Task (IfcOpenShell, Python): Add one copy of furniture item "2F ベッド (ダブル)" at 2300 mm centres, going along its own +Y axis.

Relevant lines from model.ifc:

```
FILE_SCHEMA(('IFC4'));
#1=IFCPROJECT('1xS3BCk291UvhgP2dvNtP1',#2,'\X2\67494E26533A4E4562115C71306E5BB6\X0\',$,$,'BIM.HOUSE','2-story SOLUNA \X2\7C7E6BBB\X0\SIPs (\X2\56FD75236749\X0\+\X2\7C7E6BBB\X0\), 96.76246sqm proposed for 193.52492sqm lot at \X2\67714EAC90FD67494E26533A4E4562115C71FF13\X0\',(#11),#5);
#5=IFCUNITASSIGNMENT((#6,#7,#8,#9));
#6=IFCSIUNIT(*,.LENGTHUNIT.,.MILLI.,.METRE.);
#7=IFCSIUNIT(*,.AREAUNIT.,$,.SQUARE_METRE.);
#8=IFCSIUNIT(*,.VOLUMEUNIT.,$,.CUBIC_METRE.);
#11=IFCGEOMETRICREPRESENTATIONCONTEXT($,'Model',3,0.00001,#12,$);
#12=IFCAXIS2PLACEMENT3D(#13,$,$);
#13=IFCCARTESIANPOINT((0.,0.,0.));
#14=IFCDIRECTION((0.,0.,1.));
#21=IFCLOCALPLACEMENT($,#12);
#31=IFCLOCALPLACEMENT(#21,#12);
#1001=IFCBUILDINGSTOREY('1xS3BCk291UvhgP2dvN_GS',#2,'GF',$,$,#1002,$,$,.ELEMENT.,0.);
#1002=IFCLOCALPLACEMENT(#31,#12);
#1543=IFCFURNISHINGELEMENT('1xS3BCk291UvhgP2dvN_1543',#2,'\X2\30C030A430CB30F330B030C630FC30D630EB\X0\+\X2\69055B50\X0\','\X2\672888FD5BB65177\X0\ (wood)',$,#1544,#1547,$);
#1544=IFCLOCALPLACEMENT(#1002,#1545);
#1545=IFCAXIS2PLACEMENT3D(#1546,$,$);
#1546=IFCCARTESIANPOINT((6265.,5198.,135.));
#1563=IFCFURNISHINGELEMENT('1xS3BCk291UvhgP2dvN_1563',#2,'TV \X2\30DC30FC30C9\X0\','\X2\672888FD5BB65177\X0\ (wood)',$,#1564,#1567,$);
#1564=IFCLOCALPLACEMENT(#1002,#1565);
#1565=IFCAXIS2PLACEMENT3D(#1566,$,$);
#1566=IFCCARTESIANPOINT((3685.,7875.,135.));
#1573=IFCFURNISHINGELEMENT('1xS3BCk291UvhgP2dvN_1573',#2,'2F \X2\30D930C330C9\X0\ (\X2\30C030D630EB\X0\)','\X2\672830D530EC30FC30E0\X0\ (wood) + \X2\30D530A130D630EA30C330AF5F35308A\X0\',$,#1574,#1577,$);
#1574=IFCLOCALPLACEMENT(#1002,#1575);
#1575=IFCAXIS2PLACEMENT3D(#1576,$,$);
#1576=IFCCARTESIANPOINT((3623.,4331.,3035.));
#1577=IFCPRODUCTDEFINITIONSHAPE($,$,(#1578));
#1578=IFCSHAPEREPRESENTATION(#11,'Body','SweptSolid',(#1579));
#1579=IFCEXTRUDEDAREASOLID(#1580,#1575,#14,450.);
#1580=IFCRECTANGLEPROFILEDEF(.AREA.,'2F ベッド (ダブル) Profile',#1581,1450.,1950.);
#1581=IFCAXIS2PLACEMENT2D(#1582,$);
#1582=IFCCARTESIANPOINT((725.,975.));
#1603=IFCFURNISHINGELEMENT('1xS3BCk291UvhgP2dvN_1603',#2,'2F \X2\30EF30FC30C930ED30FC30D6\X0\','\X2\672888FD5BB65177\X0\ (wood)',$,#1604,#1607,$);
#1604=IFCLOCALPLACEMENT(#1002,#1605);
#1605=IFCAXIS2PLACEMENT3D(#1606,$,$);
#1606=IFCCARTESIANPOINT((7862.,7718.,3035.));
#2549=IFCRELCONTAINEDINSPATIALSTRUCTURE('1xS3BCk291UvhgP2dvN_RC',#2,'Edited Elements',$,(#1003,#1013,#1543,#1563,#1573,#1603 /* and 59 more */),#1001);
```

```python
import ifcopenshell
import ifcopenshell.api.geometry
import ifcopenshell.api.root
import ifcopenshell.util.element
import ifcopenshell.util.placement
import ifcopenshell.util.unit

model = ifcopenshell.open("model.ifc")
unit_scale = ifcopenshell.util.unit.calculate_unit_scale(model)


def reuse_history(source, copy):
    """copy_class also copies each property set's owner history, people and application; keep the originals."""
    for rel in copy.IsDefinedBy:
        if rel.is_a("IfcRelDefinesByProperties") and (history := rel.RelatingPropertyDefinition.OwnerHistory):
            rel.RelatingPropertyDefinition.OwnerHistory = source.OwnerHistory
            ifcopenshell.util.element.remove_deep2(model, history)


source = model.by_guid("1xS3BCk291UvhgP2dvN_1573")
base = ifcopenshell.util.placement.get_local_placement(source.ObjectPlacement)
step = base[:3, 1] * 2.3 / unit_scale

for i in range(1, 2):
    copy = ifcopenshell.api.root.copy_class(model, product=source)
    copy.Representation = ifcopenshell.util.element.copy_deep(
        model, source.Representation, exclude=["IfcGeometricRepresentationContext", "IfcRepresentationMap"]
    )
    reuse_history(source, copy)
    matrix = base.copy()
    matrix[:3, 3] += i * step
    print("added at", matrix[:3, 3].round(3) + 0.0)
    ifcopenshell.api.geometry.edit_object_placement(model, product=copy, matrix=matrix, is_si=False)

model.write("model_updated.ifc")
```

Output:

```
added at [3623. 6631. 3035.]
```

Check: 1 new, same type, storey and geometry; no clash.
